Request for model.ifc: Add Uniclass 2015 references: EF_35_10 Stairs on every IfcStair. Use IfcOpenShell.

First a look at what the model holds.

```python
import ifcopenshell

model = ifcopenshell.open("model.ifc")
print(model.schema)
print("classifications:", [c.Name for c in model.by_type("IfcClassification")])
for ifc_class in ("IfcDoor", "IfcRoof", "IfcStair", "IfcWall", "IfcWindow"):
    print(ifc_class, len(model.by_type(ifc_class)))
```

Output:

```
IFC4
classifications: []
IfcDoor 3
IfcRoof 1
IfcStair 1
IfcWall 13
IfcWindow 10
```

```python
import ifcopenshell
import ifcopenshell.api.classification

model = ifcopenshell.open("model.ifc")

system = ifcopenshell.api.classification.add_classification(model, classification="Uniclass 2015")

codes = {
    "IfcStair": ("EF_35_10", "Stairs"),
}
for ifc_class, (code, name) in codes.items():
    products = model.by_type(ifc_class)
    ifcopenshell.api.classification.add_reference(
        model, products=products, classification=system, identification=code, name=name
    )
    print(code, len(products))

model.write("model_rev.ifc")
```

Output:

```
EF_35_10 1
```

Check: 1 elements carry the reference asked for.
